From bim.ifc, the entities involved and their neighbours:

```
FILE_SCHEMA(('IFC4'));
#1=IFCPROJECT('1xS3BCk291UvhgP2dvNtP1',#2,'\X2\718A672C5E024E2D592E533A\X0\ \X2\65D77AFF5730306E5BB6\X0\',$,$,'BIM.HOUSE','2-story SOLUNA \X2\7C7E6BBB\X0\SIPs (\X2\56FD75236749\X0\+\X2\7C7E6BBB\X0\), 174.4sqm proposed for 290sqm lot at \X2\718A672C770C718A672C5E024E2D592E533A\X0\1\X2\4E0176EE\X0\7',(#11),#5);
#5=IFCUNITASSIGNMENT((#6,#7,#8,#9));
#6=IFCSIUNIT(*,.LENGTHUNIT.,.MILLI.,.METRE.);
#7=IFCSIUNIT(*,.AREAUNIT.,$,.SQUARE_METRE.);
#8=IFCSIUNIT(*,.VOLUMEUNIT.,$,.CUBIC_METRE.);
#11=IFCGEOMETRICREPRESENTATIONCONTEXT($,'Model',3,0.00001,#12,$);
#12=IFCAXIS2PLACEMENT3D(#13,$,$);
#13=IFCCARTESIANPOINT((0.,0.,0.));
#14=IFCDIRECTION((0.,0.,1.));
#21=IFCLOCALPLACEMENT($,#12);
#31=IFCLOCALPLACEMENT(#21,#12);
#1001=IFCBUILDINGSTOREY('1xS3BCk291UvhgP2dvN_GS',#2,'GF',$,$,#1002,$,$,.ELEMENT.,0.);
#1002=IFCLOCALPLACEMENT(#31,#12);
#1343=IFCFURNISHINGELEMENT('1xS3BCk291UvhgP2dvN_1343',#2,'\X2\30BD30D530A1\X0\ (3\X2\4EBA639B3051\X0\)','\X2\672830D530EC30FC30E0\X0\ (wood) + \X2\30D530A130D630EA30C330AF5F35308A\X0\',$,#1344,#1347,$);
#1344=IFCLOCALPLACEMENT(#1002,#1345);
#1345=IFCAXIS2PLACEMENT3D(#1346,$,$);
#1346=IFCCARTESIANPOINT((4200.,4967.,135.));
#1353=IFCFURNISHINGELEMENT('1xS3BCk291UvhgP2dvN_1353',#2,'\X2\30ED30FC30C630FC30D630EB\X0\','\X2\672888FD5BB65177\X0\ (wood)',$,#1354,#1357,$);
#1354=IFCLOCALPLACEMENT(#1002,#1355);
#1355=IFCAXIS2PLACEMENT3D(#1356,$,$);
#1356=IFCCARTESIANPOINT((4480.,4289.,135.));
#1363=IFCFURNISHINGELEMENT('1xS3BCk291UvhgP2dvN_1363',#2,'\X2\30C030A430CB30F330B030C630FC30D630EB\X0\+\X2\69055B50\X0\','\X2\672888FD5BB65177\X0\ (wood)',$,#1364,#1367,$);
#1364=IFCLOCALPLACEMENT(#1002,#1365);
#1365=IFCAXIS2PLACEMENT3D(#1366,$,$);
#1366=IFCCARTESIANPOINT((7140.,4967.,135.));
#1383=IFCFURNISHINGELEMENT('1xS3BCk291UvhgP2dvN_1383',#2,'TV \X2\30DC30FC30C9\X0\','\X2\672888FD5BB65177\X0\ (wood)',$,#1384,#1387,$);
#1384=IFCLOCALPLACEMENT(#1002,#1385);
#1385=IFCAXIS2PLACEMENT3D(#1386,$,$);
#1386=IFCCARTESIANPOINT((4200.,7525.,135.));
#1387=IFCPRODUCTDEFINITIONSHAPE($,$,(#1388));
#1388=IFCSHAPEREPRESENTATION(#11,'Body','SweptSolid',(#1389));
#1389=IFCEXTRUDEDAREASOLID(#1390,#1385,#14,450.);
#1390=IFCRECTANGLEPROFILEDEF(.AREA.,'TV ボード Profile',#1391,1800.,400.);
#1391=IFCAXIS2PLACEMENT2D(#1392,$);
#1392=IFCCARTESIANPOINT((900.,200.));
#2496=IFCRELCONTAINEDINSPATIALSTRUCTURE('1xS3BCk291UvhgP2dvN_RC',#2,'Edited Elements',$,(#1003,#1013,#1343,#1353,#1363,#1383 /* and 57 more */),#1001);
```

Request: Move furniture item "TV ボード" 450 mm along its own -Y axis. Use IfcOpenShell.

```python
import ifcopenshell
import ifcopenshell.api.geometry
import ifcopenshell.util.placement

model = ifcopenshell.open("bim.ifc")

item = model.by_guid("1xS3BCk291UvhgP2dvN_1383")
matrix = ifcopenshell.util.placement.get_local_placement(item.ObjectPlacement)
matrix[:3, 3] -= matrix[:3, 1] * 450.0
ifcopenshell.api.geometry.edit_object_placement(model, product=item, matrix=matrix, is_si=False)

print(ifcopenshell.util.placement.get_local_placement(item.ObjectPlacement).round(3) + 0.0)

model.write("bim-out.ifc")
```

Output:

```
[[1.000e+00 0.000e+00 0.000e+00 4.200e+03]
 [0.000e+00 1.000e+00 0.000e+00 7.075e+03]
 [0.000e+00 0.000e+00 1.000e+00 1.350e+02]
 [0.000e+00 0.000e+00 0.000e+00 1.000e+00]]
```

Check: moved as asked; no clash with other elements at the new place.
